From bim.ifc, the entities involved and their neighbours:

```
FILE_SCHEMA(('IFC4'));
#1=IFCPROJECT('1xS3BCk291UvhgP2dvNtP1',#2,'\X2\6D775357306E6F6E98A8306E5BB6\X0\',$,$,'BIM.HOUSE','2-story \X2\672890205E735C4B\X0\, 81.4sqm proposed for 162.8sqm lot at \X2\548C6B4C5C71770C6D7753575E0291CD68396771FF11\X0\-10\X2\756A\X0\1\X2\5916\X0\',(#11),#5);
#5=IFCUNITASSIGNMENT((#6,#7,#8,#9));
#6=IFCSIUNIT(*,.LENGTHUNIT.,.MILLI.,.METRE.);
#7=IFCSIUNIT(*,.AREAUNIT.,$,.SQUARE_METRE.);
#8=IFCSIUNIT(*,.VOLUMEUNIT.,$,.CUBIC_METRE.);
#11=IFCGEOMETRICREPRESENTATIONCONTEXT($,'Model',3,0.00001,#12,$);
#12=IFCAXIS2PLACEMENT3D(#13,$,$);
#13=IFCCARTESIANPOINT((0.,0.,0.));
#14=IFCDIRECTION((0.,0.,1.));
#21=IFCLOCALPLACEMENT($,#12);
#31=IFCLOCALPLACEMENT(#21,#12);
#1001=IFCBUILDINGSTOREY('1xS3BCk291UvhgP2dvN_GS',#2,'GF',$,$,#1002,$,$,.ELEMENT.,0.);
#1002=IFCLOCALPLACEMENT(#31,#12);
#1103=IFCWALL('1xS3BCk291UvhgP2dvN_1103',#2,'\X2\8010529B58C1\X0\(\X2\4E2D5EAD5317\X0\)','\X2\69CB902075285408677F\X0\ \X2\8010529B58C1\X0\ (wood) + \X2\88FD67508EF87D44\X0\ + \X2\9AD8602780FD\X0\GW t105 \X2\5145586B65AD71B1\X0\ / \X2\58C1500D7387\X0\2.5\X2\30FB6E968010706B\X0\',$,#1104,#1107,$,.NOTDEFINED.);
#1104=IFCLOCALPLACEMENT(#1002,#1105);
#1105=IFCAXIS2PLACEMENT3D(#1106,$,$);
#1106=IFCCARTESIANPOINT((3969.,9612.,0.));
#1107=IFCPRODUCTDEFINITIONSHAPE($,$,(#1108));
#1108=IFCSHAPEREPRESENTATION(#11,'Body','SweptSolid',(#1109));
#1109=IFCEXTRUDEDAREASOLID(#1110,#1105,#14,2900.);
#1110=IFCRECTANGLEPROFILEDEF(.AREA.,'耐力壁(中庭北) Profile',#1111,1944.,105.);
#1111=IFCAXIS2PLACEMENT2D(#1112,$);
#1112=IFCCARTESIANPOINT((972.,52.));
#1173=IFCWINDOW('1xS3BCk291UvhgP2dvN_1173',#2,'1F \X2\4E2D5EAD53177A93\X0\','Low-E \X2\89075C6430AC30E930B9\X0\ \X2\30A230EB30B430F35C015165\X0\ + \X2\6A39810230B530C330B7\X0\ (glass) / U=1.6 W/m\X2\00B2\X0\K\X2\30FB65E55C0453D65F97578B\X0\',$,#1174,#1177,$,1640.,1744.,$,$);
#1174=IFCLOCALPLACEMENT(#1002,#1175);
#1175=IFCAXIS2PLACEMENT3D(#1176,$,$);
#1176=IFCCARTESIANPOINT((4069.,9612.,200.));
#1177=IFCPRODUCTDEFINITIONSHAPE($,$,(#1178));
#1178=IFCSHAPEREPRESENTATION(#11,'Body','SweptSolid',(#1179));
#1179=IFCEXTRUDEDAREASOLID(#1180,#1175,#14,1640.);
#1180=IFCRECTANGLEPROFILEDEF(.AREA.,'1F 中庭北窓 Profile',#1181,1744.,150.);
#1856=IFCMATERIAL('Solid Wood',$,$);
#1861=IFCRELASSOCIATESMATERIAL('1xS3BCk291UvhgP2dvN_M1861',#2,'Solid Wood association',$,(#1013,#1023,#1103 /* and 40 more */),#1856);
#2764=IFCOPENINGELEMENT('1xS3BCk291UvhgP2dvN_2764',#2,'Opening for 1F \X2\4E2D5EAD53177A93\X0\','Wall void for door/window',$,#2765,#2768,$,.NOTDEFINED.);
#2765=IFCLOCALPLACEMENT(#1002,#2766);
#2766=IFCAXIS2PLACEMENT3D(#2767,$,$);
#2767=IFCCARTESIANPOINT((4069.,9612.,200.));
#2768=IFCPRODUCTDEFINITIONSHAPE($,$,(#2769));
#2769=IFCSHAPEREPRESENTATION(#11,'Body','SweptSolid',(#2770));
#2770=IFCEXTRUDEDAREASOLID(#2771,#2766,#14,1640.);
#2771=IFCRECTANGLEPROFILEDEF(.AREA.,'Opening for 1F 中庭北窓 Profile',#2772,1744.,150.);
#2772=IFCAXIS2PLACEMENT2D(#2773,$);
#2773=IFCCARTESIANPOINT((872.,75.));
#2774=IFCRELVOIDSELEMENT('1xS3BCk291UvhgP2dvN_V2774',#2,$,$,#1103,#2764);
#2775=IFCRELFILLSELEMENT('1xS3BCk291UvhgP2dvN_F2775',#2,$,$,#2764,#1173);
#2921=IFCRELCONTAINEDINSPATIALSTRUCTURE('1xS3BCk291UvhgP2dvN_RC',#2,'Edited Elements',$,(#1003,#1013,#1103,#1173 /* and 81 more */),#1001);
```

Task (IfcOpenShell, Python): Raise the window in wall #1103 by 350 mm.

```python
import numpy as np
import ifcopenshell
import ifcopenshell.api.geometry
import ifcopenshell.util.placement
import ifcopenshell.util.unit

model = ifcopenshell.open("bim.ifc")
unit_scale = ifcopenshell.util.unit.calculate_unit_scale(model)

window = model.by_id(1173)
opening = window.FillsVoids[0].RelatingOpeningElement
dz = 0.35 / unit_scale

shift = np.array([0.0, 0.0, dz])
# The window is not placed relative to its opening, so move both.
for product in (opening, window):
    matrix = ifcopenshell.util.placement.get_local_placement(product.ObjectPlacement)
    matrix[:3, 3] += shift
    ifcopenshell.api.geometry.edit_object_placement(model, product=product, matrix=matrix, is_si=False)

print(f"moved by {dz * unit_scale:+.3f} m")

model.write("bim_rev.ifc")
```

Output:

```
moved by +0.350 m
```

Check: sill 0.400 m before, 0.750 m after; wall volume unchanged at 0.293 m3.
